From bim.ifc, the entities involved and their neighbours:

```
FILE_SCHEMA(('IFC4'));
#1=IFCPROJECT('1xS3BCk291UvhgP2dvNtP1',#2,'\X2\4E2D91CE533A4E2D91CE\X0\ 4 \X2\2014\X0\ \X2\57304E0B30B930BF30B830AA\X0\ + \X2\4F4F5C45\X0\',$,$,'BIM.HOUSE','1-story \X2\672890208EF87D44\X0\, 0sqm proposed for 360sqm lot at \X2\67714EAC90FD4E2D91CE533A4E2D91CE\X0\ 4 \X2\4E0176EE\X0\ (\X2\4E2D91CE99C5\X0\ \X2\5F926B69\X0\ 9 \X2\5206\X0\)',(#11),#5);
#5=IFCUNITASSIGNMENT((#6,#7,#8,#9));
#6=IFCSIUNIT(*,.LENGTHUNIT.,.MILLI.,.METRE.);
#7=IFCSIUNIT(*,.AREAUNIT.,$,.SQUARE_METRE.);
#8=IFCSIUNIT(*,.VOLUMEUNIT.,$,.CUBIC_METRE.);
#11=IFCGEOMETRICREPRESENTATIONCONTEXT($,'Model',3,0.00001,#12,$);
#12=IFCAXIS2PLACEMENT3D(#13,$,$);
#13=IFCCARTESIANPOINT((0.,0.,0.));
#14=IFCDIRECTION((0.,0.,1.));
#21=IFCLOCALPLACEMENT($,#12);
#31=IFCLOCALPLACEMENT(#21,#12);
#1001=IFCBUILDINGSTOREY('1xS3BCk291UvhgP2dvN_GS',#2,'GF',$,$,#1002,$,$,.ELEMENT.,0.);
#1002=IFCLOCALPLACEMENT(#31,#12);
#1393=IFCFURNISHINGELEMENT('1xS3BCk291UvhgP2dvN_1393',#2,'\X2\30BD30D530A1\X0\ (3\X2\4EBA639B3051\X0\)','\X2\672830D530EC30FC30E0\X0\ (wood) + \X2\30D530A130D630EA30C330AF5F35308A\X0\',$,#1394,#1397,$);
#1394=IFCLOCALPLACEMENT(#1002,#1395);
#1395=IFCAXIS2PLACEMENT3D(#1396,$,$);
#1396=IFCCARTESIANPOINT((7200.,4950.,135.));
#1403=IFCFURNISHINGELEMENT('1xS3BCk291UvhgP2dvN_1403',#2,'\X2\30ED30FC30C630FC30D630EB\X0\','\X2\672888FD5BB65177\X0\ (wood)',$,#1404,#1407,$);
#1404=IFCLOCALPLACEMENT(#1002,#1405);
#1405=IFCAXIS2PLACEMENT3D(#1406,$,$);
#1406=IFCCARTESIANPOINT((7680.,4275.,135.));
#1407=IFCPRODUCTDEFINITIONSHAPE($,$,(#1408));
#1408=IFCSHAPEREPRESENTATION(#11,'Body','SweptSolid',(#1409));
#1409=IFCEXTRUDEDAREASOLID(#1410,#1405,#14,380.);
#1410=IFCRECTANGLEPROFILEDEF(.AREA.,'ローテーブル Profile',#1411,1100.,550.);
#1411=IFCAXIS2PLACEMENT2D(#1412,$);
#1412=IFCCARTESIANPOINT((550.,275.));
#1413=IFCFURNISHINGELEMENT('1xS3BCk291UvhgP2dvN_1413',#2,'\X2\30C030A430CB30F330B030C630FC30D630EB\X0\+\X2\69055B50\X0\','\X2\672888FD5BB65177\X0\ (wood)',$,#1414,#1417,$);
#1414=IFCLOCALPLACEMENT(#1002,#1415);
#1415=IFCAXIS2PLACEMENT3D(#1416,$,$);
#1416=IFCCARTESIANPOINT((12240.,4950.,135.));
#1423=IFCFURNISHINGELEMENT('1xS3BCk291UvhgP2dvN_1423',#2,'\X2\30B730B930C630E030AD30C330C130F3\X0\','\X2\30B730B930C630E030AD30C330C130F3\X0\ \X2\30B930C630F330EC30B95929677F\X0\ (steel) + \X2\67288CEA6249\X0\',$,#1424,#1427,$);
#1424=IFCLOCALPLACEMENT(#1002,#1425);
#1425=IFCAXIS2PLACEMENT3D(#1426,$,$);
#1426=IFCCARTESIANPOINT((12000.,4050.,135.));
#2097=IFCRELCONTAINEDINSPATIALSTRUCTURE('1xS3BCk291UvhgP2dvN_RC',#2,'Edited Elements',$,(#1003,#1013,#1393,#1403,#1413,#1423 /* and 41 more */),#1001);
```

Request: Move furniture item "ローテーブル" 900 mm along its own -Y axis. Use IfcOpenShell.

```python
import ifcopenshell
import ifcopenshell.api.geometry
import ifcopenshell.util.placement

model = ifcopenshell.open("bim.ifc")

item = model.by_guid("1xS3BCk291UvhgP2dvN_1403")
matrix = ifcopenshell.util.placement.get_local_placement(item.ObjectPlacement)
matrix[:3, 3] -= matrix[:3, 1] * 900.0
ifcopenshell.api.geometry.edit_object_placement(model, product=item, matrix=matrix, is_si=False)

print(ifcopenshell.util.placement.get_local_placement(item.ObjectPlacement).round(3) + 0.0)

model.write("bim_v2.ifc")
```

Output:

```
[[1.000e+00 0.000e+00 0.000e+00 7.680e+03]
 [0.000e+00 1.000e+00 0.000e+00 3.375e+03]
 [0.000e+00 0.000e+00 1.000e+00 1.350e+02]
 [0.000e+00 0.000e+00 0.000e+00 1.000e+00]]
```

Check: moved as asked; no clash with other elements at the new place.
